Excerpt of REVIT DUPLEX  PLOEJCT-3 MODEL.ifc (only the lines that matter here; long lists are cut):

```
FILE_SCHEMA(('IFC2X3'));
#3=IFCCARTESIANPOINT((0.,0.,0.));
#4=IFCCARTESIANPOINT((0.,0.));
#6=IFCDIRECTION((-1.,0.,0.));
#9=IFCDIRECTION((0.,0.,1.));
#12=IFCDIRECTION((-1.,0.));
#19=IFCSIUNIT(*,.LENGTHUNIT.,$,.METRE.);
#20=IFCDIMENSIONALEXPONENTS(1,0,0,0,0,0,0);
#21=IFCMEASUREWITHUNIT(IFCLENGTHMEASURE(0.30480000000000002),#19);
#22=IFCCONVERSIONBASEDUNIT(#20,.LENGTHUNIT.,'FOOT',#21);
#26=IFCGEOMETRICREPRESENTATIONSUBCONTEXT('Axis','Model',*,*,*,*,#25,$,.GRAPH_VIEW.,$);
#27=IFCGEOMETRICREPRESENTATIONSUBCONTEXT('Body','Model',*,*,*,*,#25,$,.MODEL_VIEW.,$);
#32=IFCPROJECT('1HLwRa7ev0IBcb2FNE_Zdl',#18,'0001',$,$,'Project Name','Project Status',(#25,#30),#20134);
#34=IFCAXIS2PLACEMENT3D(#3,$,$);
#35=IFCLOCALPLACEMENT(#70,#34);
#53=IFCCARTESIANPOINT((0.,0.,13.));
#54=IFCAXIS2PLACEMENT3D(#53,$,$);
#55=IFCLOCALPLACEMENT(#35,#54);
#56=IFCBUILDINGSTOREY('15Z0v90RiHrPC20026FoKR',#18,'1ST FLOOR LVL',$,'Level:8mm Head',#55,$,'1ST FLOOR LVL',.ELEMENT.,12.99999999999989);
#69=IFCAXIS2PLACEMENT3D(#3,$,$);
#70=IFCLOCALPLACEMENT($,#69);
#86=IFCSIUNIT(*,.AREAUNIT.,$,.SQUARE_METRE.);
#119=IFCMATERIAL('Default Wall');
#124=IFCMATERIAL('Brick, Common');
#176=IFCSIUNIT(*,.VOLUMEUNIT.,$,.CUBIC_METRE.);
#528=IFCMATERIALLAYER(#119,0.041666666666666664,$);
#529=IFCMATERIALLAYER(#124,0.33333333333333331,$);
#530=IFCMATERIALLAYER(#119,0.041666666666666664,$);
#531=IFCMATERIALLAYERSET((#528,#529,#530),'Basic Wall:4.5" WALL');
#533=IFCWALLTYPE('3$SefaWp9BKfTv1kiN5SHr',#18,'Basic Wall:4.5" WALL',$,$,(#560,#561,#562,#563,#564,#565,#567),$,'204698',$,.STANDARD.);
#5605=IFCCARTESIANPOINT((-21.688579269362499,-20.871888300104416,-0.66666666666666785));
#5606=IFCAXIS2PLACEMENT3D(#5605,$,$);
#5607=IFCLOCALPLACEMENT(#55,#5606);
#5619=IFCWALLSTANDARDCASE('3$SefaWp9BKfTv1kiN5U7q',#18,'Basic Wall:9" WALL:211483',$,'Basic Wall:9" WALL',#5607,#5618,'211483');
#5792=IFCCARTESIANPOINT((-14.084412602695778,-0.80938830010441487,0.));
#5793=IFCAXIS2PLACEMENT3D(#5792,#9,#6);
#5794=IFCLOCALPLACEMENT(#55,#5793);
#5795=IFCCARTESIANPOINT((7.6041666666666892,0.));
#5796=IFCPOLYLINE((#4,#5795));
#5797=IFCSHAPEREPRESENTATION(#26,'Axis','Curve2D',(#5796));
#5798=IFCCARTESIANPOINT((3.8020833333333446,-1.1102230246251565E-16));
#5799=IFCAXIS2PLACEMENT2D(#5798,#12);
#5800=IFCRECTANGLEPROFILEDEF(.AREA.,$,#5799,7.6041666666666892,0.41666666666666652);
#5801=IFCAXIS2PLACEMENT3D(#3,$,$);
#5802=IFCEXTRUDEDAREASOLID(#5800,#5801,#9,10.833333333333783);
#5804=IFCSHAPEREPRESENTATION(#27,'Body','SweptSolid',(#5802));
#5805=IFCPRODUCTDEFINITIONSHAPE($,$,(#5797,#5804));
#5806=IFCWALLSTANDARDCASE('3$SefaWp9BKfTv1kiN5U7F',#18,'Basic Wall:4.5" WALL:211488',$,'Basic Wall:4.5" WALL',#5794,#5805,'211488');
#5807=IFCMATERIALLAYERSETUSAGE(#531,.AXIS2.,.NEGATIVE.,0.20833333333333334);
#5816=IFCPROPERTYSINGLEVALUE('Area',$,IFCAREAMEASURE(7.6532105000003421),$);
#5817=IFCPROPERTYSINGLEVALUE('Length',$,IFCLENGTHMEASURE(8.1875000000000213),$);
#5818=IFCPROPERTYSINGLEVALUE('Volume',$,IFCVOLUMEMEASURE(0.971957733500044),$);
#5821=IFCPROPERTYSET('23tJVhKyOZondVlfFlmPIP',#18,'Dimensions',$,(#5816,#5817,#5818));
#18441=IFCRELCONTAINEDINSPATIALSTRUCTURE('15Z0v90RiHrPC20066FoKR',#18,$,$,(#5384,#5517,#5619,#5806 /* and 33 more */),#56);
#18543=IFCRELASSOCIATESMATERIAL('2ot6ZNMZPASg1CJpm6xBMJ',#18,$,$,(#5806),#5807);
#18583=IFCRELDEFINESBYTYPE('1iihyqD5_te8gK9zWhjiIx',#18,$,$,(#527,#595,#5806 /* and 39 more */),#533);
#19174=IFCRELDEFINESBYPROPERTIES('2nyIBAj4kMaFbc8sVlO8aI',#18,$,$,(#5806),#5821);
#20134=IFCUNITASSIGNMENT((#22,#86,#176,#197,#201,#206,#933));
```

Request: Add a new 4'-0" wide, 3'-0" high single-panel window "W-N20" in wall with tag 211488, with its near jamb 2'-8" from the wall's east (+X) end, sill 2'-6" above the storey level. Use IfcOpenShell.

```python
import numpy as np
import ifcopenshell
import ifcopenshell.api.feature
import ifcopenshell.api.geometry
import ifcopenshell.api.pset
import ifcopenshell.api.root
import ifcopenshell.api.spatial
import ifcopenshell.api.type
import ifcopenshell.geom
import ifcopenshell.util.element
import ifcopenshell.util.placement
import ifcopenshell.util.representation
import ifcopenshell.util.shape
import ifcopenshell.util.unit

model = ifcopenshell.open("REVIT DUPLEX  PLOEJCT-3 MODEL.ifc")
unit_scale = ifcopenshell.util.unit.calculate_unit_scale(model)
area_scale = ifcopenshell.util.unit.calculate_unit_scale(model, "AREAUNIT")
volume_scale = ifcopenshell.util.unit.calculate_unit_scale(model, "VOLUMEUNIT")
settings = ifcopenshell.geom.settings()


def volume(element):
    """Net volume in cubic metres, openings subtracted."""
    shape = ifcopenshell.geom.create_shape(settings, element)
    return ifcopenshell.util.shape.get_volume(shape.geometry)


wall = model.by_id(5806)
storey = ifcopenshell.util.element.get_container(wall, ifc_class="IfcBuildingStorey")
context = ifcopenshell.util.representation.get_context(model, "Model", "Body", "MODEL_VIEW")
before = volume(wall)

width, height, from_end, sill = 1.2192, 0.9144, 0.8128, 0.762  # metres

# The wall runs along its own X axis, and the end named is its -X end.
wall_shape = ifcopenshell.geom.create_shape(settings, wall)
x, y, z = ifcopenshell.util.shape.get_vertices(wall_shape.geometry).T
start = x.min() + from_end
face, thickness = float(y.min()), float(y.max() - y.min())
wall_matrix = ifcopenshell.util.placement.get_local_placement(wall.ObjectPlacement)
level = ifcopenshell.util.placement.get_local_placement(storey.ObjectPlacement)[2, 3]


def in_wall(x, y):
    """Placement at x, y metres in the wall's axes, at sill height."""
    matrix = wall_matrix.copy()
    matrix[:, 3] = wall_matrix @ np.array([x / unit_scale, y / unit_scale, 0.0, 1.0])
    matrix[2, 3] = level + sill / unit_scale
    return matrix


# Opening: a box that overshoots both wall faces by 50 mm.
opening = ifcopenshell.api.root.create_entity(model, ifc_class="IfcOpeningElement")
box = ifcopenshell.api.geometry.add_wall_representation(
    model, context=context, length=width, height=height, thickness=thickness + 0.1
)
ifcopenshell.api.geometry.assign_representation(model, product=opening, representation=box)
ifcopenshell.api.geometry.edit_object_placement(model, product=opening, matrix=in_wall(start, face - 0.05), is_si=False)
ifcopenshell.api.feature.add_feature(model, feature=opening, element=wall)

window = ifcopenshell.api.root.create_entity(model, ifc_class="IfcWindow", name="W-N20")
window.OverallWidth, window.OverallHeight = width / unit_scale, height / unit_scale
body = ifcopenshell.api.geometry.add_window_representation(
    model,
    context=context,
    overall_width=window.OverallWidth,
    overall_height=window.OverallHeight,
    partition_type="SINGLE_PANEL",
)
ifcopenshell.api.geometry.assign_representation(model, product=window, representation=body)
ifcopenshell.api.spatial.assign_container(model, products=[window], relating_structure=storey)
fills = ifcopenshell.api.feature.add_filling(model, opening=opening, element=window)
fills.OwnerHistory = window.OwnerHistory  # required in IFC2X3

# IFC2X3 keeps the operation on the window style.
style = ifcopenshell.api.root.create_entity(model, ifc_class="IfcWindowStyle", name="W-N20")
style.OperationType, style.ConstructionType = "SINGLE_PANEL", "NOTDEFINED"
style.ParameterTakesPrecedence = style.Sizeable = False
ifcopenshell.api.type.assign_type(model, related_objects=[window], relating_type=style)

# Centre the window in the wall's thickness.
ifcopenshell.api.geometry.edit_object_placement(model, product=window, matrix=in_wall(start, face), is_si=False)
window_shape = ifcopenshell.geom.create_shape(settings, window)
depth = ifcopenshell.util.shape.get_vertices(window_shape.geometry)[:, 1]
offset = face + thickness / 2 - (depth.min() + depth.max()) / 2
ifcopenshell.api.geometry.edit_object_placement(model, product=window, matrix=in_wall(start, offset), is_si=False)

after = volume(wall)

# Update the wall's stored quantities.
pset = model.by_id(ifcopenshell.util.element.get_pset(wall, "Dimensions", should_inherit=False)["id"])
ifcopenshell.api.pset.edit_pset(model, pset=pset, properties={
    "Area": model.create_entity("IfcAreaMeasure", after / thickness / area_scale),
    "Volume": model.create_entity("IfcVolumeMeasure", after / volume_scale),
})

print(f"wall volume {before:.3f} -> {after:.3f} m3")

model.write("REVIT DUPLEX  PLOEJCT-3 MODEL_rev.ifc")
```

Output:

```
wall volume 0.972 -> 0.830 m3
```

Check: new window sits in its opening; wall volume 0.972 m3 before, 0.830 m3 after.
